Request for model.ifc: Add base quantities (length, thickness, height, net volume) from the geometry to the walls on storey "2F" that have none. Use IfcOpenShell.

First a look at what the model holds.

```python
import ifcopenshell
import ifcopenshell.util.element
import ifcopenshell.util.unit

model = ifcopenshell.open("model.ifc")
print(model.schema)
for unit_type in ("LENGTHUNIT", "AREAUNIT", "VOLUMEUNIT"):
    print(unit_type, ifcopenshell.util.unit.calculate_unit_scale(model, unit_type))
storey = next(s for s in model.by_type("IfcBuildingStorey") if s.Name == "2F")
walls = [e for e in ifcopenshell.util.element.get_decomposition(storey) if e.is_a("IfcWall")]
for e in sorted(walls, key=lambda e: e.id()):
    print(e.id(), e.is_a(), e.Name, list(ifcopenshell.util.element.get_psets(e, qtos_only=True)), sep=" | ")
```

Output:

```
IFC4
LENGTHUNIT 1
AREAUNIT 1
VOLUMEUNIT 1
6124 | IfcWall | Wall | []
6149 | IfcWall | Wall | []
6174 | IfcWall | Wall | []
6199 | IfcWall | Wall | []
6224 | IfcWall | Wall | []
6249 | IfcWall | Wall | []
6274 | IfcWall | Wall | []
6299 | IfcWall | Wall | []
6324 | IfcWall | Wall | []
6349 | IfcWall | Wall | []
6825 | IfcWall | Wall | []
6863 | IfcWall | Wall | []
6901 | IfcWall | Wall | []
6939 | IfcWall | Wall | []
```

```python
import ifcopenshell
import ifcopenshell.api.pset
import ifcopenshell.geom
import ifcopenshell.util.element
import ifcopenshell.util.shape
import ifcopenshell.util.unit

model = ifcopenshell.open("model.ifc")
unit_scale = ifcopenshell.util.unit.calculate_unit_scale(model)
volume_scale = ifcopenshell.util.unit.calculate_unit_scale(model, "VOLUMEUNIT")
settings = ifcopenshell.geom.settings()

storey = next(s for s in model.by_type("IfcBuildingStorey") if s.Name == "2F")
walls = [e for e in ifcopenshell.util.element.get_decomposition(storey) if e.is_a("IfcWall")]

for e in sorted(walls, key=lambda e: e.id()):
    if ifcopenshell.util.element.get_psets(e, qtos_only=True, should_inherit=False):
        continue
    # Geometry comes back in metres, in the element's own axes.
    shape = ifcopenshell.geom.create_shape(settings, e)
    values = {
        "Length": ifcopenshell.util.shape.get_x(shape.geometry) / unit_scale,
        "Width": ifcopenshell.util.shape.get_y(shape.geometry) / unit_scale,
        "Height": ifcopenshell.util.shape.get_z(shape.geometry) / unit_scale,
        "NetVolume": ifcopenshell.util.shape.get_volume(shape.geometry) / volume_scale,
    }
    qto = ifcopenshell.api.pset.add_qto(model, product=e, name="Qto_WallBaseQuantities")
    ifcopenshell.api.pset.edit_qto(model, qto=qto, properties=values)
    print(e.id(), {k: round(v, 3) for k, v in values.items()})

model.write("model-out.ifc")
```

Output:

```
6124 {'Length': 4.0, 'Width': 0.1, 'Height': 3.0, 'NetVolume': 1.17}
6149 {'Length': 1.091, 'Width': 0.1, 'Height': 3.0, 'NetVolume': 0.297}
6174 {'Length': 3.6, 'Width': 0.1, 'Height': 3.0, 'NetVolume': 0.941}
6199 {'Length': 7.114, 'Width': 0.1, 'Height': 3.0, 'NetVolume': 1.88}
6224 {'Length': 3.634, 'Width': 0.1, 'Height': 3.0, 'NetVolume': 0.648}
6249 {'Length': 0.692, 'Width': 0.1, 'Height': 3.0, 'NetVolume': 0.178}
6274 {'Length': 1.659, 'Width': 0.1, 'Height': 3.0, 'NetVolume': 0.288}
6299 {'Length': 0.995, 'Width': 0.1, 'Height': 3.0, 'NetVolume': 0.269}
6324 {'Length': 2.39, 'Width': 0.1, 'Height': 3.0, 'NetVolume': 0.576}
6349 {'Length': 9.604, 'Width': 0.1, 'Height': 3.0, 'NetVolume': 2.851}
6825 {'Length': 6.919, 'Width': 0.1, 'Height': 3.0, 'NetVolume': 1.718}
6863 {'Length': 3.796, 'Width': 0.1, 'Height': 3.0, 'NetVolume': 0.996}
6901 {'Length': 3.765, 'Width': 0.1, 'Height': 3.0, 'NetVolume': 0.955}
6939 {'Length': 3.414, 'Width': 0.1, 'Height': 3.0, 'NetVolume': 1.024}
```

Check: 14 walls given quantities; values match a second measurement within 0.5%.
